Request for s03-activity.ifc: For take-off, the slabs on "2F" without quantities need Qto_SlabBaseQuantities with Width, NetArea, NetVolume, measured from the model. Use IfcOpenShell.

First a look at what the model holds.

```python
import ifcopenshell
import ifcopenshell.util.element
import ifcopenshell.util.unit

model = ifcopenshell.open("s03-activity.ifc")
print(model.schema)
for unit_type in ("LENGTHUNIT", "AREAUNIT", "VOLUMEUNIT"):
    print(unit_type, ifcopenshell.util.unit.calculate_unit_scale(model, unit_type))
storey = next(s for s in model.by_type("IfcBuildingStorey") if s.Name == "2F")
slabs = [e for e in ifcopenshell.util.element.get_decomposition(storey) if e.is_a("IfcSlab")]
for e in sorted(slabs, key=lambda e: e.id()):
    print(e.id(), e.is_a(), e.Name, list(ifcopenshell.util.element.get_psets(e, qtos_only=True)), sep=" | ")
```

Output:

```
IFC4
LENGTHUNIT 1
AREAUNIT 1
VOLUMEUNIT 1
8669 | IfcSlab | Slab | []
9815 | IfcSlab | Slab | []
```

```python
import ifcopenshell
import ifcopenshell.api.pset
import ifcopenshell.geom
import ifcopenshell.util.element
import ifcopenshell.util.shape
import ifcopenshell.util.unit

model = ifcopenshell.open("s03-activity.ifc")
unit_scale = ifcopenshell.util.unit.calculate_unit_scale(model)
area_scale = ifcopenshell.util.unit.calculate_unit_scale(model, "AREAUNIT")
volume_scale = ifcopenshell.util.unit.calculate_unit_scale(model, "VOLUMEUNIT")
settings = ifcopenshell.geom.settings()

storey = next(s for s in model.by_type("IfcBuildingStorey") if s.Name == "2F")
slabs = [e for e in ifcopenshell.util.element.get_decomposition(storey) if e.is_a("IfcSlab")]

for e in sorted(slabs, key=lambda e: e.id()):
    if ifcopenshell.util.element.get_psets(e, qtos_only=True, should_inherit=False):
        continue
    # Geometry comes back in metres, in the element's own axes.
    shape = ifcopenshell.geom.create_shape(settings, e)
    values = {
        "Width": ifcopenshell.util.shape.get_z(shape.geometry) / unit_scale,
        "NetArea": ifcopenshell.util.shape.get_footprint_area(shape.geometry) / area_scale,
        "NetVolume": ifcopenshell.util.shape.get_volume(shape.geometry) / volume_scale,
    }
    qto = ifcopenshell.api.pset.add_qto(model, product=e, name="Qto_SlabBaseQuantities")
    ifcopenshell.api.pset.edit_qto(model, qto=qto, properties=values)
    print(e.id(), {k: round(v, 3) for k, v in values.items()})

model.write("s03-activity-out.ifc")
```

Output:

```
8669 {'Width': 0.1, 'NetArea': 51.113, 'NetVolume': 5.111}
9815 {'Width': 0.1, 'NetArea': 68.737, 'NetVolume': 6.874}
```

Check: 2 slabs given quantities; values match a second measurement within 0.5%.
